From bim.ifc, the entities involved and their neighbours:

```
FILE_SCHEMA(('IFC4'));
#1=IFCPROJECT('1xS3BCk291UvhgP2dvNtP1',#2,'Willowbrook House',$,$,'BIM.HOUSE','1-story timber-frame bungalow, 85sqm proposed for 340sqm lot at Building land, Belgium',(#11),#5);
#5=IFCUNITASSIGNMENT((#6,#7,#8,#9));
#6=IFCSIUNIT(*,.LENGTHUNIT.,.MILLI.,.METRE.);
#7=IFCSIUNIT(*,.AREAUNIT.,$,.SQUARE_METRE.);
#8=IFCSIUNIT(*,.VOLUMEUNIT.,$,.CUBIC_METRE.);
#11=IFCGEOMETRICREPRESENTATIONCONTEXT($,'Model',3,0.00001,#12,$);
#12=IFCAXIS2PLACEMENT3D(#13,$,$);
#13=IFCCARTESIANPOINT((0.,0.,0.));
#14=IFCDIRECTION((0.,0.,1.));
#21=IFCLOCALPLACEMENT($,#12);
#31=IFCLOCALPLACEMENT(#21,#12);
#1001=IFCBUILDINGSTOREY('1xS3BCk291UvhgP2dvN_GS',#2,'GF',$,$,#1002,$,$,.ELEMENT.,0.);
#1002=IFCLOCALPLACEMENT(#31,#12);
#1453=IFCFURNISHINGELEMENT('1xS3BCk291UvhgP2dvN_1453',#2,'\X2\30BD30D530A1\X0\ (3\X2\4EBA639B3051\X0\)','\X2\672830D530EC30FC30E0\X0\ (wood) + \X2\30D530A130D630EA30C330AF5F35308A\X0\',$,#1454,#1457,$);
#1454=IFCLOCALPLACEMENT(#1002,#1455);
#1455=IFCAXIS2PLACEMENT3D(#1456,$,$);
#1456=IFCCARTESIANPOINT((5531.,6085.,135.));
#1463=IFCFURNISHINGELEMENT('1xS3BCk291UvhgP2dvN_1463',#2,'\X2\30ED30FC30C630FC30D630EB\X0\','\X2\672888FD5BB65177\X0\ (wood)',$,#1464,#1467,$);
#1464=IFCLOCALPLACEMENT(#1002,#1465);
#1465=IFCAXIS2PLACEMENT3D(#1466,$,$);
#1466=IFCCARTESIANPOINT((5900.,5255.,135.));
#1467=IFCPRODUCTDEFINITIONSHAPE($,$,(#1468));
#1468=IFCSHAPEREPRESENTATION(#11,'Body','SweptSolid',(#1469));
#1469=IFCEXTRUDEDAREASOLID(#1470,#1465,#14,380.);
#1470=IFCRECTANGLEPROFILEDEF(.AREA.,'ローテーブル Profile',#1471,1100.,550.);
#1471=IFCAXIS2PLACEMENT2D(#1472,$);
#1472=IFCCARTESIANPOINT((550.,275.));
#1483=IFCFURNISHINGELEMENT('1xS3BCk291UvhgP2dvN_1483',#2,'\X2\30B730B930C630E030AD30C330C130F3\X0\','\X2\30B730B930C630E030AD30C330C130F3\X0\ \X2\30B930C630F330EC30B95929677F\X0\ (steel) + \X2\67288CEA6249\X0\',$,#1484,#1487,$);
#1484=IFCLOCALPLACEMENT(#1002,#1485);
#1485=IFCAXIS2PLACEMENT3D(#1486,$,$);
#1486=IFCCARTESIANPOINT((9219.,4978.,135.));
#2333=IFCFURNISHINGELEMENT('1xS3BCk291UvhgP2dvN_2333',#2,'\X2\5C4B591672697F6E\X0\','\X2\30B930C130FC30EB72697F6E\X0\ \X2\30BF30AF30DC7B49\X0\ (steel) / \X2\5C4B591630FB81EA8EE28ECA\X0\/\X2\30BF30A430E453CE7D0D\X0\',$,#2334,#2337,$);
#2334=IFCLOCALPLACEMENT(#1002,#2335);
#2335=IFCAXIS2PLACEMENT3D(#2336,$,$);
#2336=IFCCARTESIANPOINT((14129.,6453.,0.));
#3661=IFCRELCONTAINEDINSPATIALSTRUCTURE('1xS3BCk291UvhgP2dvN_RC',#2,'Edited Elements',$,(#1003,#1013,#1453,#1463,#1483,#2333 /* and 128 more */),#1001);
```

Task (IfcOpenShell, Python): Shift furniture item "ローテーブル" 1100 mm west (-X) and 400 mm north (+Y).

```python
import ifcopenshell
import ifcopenshell.api.geometry
import ifcopenshell.util.placement

model = ifcopenshell.open("bim.ifc")

item = model.by_guid("1xS3BCk291UvhgP2dvN_1463")
matrix = ifcopenshell.util.placement.get_local_placement(item.ObjectPlacement)
matrix[0, 3] -= 1100.0
matrix[1, 3] += 400.0
ifcopenshell.api.geometry.edit_object_placement(model, product=item, matrix=matrix, is_si=False)

print(ifcopenshell.util.placement.get_local_placement(item.ObjectPlacement).round(3) + 0.0)

model.write("bim-out.ifc")
```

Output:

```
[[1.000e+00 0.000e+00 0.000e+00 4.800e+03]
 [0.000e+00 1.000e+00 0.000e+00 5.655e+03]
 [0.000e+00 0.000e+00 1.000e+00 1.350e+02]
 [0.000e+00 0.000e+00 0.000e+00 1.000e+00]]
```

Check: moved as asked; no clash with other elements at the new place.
